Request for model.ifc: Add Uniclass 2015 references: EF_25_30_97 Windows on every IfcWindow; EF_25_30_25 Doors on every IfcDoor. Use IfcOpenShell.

First a look at what the model holds.

```python
import ifcopenshell

model = ifcopenshell.open("model.ifc")
print(model.schema)
print("classifications:", [c.Name for c in model.by_type("IfcClassification")])
for ifc_class in ("IfcDoor", "IfcRoof", "IfcStair", "IfcWall", "IfcWindow"):
    print(ifc_class, len(model.by_type(ifc_class)))
```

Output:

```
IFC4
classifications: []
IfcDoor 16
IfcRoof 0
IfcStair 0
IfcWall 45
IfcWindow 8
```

```python
import ifcopenshell
import ifcopenshell.api.classification

model = ifcopenshell.open("model.ifc")

system = ifcopenshell.api.classification.add_classification(model, classification="Uniclass 2015")

codes = {
    "IfcWindow": ("EF_25_30_97", "Windows"),
    "IfcDoor": ("EF_25_30_25", "Doors"),
}
for ifc_class, (code, name) in codes.items():
    products = model.by_type(ifc_class)
    ifcopenshell.api.classification.add_reference(
        model, products=products, classification=system, identification=code, name=name
    )
    print(code, len(products))

model.write("model_rev.ifc")
```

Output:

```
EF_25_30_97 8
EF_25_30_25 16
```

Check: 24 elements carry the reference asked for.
